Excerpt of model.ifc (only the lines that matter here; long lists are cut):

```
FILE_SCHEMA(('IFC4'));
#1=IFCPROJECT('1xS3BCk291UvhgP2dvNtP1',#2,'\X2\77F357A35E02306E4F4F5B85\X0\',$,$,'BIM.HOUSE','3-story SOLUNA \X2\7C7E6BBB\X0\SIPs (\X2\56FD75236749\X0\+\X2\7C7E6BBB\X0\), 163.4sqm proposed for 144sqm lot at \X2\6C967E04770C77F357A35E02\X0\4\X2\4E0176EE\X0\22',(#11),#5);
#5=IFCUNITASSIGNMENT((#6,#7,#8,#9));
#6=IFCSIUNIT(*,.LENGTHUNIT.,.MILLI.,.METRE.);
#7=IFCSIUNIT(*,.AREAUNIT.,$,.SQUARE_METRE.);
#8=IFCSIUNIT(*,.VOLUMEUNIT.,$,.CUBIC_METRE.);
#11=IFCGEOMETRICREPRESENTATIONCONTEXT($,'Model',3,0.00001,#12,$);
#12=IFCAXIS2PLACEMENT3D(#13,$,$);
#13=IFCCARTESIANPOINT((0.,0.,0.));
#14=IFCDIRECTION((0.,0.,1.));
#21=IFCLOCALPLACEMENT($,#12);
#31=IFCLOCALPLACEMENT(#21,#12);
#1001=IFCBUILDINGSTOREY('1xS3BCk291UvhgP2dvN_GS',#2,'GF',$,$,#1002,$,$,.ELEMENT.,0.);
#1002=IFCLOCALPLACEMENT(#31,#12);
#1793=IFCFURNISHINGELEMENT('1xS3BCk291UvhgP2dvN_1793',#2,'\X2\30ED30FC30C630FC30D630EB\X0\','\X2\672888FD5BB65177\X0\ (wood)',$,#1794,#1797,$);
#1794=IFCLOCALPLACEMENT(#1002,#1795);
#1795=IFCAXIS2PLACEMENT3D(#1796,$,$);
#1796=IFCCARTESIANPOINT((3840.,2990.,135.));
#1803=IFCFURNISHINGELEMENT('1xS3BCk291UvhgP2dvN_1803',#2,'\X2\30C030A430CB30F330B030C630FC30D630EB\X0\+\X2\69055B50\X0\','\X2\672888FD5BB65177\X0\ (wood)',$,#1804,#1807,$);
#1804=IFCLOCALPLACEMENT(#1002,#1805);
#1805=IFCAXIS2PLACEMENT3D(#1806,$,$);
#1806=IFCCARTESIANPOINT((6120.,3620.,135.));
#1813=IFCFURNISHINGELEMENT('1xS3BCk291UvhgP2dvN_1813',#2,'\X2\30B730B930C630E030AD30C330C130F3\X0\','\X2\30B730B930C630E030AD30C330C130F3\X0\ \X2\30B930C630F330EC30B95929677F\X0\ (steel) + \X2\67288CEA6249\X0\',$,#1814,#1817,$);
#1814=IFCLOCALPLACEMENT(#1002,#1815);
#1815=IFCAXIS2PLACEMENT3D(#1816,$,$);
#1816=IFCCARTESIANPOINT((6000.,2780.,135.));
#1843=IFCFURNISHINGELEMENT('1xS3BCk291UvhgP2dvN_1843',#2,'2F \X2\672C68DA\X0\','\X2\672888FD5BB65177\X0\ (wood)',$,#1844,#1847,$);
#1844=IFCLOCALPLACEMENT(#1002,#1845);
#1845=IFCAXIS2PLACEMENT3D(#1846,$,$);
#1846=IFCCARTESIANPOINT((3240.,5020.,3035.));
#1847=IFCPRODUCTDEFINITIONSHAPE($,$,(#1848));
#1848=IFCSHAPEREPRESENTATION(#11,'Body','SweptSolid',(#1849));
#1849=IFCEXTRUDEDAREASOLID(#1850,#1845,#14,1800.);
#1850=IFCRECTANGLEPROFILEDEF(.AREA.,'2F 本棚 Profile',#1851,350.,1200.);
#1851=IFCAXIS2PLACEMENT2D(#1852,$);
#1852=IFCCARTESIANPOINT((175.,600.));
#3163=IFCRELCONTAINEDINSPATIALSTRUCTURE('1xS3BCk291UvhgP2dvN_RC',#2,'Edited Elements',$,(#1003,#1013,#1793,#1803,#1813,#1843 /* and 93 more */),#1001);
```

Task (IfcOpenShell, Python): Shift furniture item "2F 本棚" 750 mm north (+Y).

```python
import ifcopenshell
import ifcopenshell.api.geometry
import ifcopenshell.util.placement

model = ifcopenshell.open("model.ifc")

item = model.by_guid("1xS3BCk291UvhgP2dvN_1843")
matrix = ifcopenshell.util.placement.get_local_placement(item.ObjectPlacement)
matrix[1, 3] += 750.0
ifcopenshell.api.geometry.edit_object_placement(model, product=item, matrix=matrix, is_si=False)

print(ifcopenshell.util.placement.get_local_placement(item.ObjectPlacement).round(3) + 0.0)

model.write("model_rev.ifc")
```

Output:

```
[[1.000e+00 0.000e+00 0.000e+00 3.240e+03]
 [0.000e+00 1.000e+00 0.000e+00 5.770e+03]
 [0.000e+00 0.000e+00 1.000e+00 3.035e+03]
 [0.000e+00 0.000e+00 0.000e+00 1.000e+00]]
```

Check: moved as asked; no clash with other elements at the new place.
